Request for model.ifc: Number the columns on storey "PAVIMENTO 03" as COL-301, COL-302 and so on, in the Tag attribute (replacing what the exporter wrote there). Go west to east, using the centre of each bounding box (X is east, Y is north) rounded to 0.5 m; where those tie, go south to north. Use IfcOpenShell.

First a look at what the model holds.

```python
import ifcopenshell
import ifcopenshell.util.element
import ifcopenshell.util.placement

model = ifcopenshell.open("model.ifc")
print(model.schema)
storey = next(s for s in model.by_type("IfcBuildingStorey") if s.Name == "PAVIMENTO 03")
columns = [e for e in ifcopenshell.util.element.get_decomposition(storey) if e.is_a("IfcColumn")]
for e in sorted(columns, key=lambda e: e.id()):
    origin = ifcopenshell.util.placement.get_local_placement(e.ObjectPlacement)[:3, 3]
    print(e.id(), e.Tag, e.Name, origin.round(2) + 0.0, sep=" | ")
```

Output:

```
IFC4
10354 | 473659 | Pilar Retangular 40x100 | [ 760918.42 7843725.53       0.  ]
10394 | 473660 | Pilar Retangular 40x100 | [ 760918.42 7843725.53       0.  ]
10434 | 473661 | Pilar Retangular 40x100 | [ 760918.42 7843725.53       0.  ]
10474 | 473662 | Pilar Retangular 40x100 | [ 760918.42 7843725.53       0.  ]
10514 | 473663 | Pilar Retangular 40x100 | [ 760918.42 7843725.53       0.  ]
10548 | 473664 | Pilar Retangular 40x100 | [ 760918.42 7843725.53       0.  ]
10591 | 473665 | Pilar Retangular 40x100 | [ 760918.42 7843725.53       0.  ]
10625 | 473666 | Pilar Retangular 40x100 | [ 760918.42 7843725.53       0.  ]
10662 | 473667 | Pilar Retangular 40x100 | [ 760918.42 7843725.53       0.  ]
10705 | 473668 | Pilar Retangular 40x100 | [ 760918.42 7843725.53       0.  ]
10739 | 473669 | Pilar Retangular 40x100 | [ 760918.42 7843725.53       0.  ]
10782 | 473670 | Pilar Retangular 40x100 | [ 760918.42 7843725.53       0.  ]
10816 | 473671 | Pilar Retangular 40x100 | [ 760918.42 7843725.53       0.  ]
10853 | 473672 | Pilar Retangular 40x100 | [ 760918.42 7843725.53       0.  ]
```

```python
import ifcopenshell
import ifcopenshell.geom
import ifcopenshell.util.element
import ifcopenshell.util.shape

model = ifcopenshell.open("model.ifc")
settings = ifcopenshell.geom.settings()
settings.set("use-world-coords", True)


def centre(element):
    shape = ifcopenshell.geom.create_shape(settings, element)
    return ifcopenshell.util.shape.get_bbox_centroid(shape.geometry)


storey = next(s for s in model.by_type("IfcBuildingStorey") if s.Name == "PAVIMENTO 03")
columns = [e for e in ifcopenshell.util.element.get_decomposition(storey) if e.is_a("IfcColumn")]

# Insertion points can sit at a corner or the storey origin, so sort by the geometry (in metres).
centres = {e: centre(e) for e in columns}
columns.sort(key=lambda e: (round(centres[e][0] / 0.5), centres[e][1]))

for i, e in enumerate(columns, start=1):
    number = f"COL-3{i:02d}"
    e.Tag = number
    print(e.id(), number)

model.write("model-out.ifc")
```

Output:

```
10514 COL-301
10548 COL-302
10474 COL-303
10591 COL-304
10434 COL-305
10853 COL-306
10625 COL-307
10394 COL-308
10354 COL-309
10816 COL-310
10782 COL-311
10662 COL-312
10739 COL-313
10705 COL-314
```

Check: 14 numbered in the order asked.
